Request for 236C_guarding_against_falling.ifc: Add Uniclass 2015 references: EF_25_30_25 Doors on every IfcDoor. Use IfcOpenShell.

First a look at what the model holds.

```python
import ifcopenshell

model = ifcopenshell.open("236C_guarding_against_falling.ifc")
print(model.schema)
print("classifications:", [c.Name for c in model.by_type("IfcClassification")])
for ifc_class in ("IfcDoor", "IfcRoof", "IfcStair", "IfcWall", "IfcWindow"):
    print(ifc_class, len(model.by_type(ifc_class)))
```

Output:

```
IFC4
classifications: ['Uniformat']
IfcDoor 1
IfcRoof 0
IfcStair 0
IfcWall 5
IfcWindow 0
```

```python
import ifcopenshell
import ifcopenshell.api.classification

model = ifcopenshell.open("236C_guarding_against_falling.ifc")

system = ifcopenshell.api.classification.add_classification(model, classification="Uniclass 2015")

codes = {
    "IfcDoor": ("EF_25_30_25", "Doors"),
}
for ifc_class, (code, name) in codes.items():
    products = model.by_type(ifc_class)
    ifcopenshell.api.classification.add_reference(
        model, products=products, classification=system, identification=code, name=name
    )
    print(code, len(products))

model.write("236C_guarding_against_falling_edited.ifc")
```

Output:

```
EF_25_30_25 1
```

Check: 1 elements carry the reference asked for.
